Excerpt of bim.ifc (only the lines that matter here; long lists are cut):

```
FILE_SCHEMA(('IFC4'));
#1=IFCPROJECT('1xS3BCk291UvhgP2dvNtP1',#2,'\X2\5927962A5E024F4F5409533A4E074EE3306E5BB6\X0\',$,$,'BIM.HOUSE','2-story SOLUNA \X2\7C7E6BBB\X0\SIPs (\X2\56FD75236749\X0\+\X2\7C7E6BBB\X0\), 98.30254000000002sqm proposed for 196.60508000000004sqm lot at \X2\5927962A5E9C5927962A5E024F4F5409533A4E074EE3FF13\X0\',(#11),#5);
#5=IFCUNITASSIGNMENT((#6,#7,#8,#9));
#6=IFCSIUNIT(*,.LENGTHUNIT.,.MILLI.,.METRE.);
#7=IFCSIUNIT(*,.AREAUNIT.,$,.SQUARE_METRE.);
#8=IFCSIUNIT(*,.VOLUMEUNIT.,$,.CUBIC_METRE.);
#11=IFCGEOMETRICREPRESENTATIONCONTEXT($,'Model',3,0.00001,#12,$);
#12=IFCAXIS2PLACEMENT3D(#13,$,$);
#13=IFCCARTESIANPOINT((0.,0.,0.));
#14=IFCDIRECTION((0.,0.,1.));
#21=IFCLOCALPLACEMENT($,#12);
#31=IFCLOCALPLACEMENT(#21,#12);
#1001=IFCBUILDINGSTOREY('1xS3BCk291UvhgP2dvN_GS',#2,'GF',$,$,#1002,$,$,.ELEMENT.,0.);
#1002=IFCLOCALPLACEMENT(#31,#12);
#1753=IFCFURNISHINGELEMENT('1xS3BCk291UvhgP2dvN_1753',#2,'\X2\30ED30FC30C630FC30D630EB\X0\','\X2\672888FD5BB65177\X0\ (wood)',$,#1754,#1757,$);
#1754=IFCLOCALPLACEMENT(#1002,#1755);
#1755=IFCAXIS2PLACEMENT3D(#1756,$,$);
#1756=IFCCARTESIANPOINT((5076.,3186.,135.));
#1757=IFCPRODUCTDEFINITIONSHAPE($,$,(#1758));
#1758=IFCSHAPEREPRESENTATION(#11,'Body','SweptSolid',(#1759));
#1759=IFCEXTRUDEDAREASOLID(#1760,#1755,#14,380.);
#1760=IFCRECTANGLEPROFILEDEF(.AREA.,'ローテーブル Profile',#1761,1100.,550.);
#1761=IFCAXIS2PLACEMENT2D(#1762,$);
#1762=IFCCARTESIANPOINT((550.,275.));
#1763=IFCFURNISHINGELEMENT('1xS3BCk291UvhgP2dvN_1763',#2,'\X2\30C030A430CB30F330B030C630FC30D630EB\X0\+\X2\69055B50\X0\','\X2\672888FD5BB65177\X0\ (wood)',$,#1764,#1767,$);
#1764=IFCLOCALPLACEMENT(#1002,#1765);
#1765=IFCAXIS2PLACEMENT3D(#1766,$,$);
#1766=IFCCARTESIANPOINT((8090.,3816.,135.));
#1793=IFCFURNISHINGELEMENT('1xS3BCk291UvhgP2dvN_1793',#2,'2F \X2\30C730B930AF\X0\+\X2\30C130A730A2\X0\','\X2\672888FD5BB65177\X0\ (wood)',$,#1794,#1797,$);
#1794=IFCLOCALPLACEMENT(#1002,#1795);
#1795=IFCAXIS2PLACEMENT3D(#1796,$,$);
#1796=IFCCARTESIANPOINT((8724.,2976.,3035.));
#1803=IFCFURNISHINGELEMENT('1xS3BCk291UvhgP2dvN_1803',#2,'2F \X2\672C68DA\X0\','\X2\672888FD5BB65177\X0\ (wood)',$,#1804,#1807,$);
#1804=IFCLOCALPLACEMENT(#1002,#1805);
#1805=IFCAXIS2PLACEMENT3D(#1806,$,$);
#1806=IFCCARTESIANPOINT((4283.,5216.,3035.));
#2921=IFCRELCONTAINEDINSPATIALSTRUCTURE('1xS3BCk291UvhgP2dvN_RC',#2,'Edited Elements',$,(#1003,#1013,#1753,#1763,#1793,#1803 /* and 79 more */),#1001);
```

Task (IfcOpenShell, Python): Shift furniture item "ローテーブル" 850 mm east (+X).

```python
import ifcopenshell
import ifcopenshell.api.geometry
import ifcopenshell.util.placement
import ifcopenshell.util.unit

model = ifcopenshell.open("bim.ifc")
unit_scale = ifcopenshell.util.unit.calculate_unit_scale(model)

item = model.by_id(1753)
matrix = ifcopenshell.util.placement.get_local_placement(item.ObjectPlacement)
matrix[0, 3] += 0.85 / unit_scale
ifcopenshell.api.geometry.edit_object_placement(model, product=item, matrix=matrix, is_si=False)

print(ifcopenshell.util.placement.get_local_placement(item.ObjectPlacement).round(3) + 0.0)

model.write("bim-out.ifc")
```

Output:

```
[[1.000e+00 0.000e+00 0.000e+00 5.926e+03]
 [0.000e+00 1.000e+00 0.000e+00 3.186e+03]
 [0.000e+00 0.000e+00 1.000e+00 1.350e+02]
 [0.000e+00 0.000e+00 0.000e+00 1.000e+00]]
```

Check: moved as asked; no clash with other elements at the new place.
